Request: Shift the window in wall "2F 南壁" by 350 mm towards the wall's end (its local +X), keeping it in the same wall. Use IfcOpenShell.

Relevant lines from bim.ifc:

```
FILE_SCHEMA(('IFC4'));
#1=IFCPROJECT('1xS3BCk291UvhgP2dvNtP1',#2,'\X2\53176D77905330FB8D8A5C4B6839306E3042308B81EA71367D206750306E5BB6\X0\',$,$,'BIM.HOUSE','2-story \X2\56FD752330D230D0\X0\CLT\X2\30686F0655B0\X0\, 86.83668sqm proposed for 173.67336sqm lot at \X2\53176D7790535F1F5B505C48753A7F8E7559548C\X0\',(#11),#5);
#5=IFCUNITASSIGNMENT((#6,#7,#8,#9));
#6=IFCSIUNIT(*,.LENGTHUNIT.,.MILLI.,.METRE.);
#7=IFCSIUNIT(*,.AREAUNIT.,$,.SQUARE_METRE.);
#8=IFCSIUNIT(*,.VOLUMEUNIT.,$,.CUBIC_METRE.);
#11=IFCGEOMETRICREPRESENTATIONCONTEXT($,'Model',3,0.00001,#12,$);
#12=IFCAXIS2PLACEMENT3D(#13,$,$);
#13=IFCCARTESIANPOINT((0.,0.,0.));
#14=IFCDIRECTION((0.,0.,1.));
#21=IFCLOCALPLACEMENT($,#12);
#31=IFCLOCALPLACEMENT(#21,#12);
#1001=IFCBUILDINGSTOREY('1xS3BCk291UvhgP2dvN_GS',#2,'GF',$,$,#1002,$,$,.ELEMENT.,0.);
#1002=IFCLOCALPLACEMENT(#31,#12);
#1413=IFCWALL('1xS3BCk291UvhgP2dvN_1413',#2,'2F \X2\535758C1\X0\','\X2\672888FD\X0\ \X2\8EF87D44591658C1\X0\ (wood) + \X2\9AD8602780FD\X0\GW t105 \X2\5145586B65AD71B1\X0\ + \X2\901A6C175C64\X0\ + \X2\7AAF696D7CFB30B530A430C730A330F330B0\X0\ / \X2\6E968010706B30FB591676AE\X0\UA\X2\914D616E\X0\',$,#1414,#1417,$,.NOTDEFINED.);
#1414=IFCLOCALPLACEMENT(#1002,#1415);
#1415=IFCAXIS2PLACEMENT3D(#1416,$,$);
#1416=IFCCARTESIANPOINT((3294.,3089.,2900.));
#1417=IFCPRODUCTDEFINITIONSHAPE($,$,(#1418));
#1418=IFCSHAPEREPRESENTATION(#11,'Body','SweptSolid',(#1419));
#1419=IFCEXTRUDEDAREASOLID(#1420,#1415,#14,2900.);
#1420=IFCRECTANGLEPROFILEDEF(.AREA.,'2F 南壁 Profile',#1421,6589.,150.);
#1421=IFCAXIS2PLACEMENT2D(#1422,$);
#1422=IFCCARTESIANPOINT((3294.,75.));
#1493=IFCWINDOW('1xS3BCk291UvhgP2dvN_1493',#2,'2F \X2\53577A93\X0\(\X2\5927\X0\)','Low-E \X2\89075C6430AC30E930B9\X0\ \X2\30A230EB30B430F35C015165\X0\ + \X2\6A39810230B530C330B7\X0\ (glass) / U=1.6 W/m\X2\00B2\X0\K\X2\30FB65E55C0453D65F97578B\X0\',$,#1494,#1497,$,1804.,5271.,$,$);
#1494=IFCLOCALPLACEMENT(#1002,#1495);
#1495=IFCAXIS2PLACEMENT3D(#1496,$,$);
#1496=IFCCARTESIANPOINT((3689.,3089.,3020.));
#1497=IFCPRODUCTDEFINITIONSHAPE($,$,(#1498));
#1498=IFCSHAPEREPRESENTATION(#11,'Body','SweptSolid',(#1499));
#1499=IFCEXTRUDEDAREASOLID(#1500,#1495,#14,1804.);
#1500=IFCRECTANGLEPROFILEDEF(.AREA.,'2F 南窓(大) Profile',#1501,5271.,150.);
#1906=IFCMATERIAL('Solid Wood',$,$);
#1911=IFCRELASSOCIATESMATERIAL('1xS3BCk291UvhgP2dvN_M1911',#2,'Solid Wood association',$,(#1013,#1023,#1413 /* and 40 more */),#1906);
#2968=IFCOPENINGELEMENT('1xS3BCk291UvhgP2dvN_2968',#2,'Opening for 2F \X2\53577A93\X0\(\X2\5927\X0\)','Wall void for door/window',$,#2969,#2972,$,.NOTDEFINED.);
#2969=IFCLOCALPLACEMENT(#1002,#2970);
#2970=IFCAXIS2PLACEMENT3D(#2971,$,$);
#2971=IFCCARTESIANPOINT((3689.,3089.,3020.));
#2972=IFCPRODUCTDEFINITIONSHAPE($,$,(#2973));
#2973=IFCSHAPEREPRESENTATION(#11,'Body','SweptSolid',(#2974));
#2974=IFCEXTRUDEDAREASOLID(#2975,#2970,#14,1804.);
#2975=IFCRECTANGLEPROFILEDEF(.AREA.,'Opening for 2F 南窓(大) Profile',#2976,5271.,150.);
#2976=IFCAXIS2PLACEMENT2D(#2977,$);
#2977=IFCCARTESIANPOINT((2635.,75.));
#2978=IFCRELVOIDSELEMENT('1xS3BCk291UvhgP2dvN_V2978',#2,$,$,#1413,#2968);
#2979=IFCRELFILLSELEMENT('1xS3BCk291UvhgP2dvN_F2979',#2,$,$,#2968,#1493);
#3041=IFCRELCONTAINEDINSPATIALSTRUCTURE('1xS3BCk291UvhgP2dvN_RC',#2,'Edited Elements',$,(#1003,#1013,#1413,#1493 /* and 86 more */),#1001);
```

```python
import ifcopenshell
import ifcopenshell.api.geometry
import ifcopenshell.util.placement
import ifcopenshell.util.unit

model = ifcopenshell.open("bim.ifc")
unit_scale = ifcopenshell.util.unit.calculate_unit_scale(model)

window = model.by_guid("1xS3BCk291UvhgP2dvN_1493")
opening = window.FillsVoids[0].RelatingOpeningElement
wall = opening.VoidsElements[0].RelatingBuildingElement

wall_matrix = ifcopenshell.util.placement.get_local_placement(wall.ObjectPlacement)
shift = wall_matrix[:3, 0] * 0.35 / unit_scale
before = ifcopenshell.util.placement.get_local_placement(window.ObjectPlacement)[:3, 3].copy()

# The window is not placed relative to its opening, so move both.
for product in (opening, window):
    matrix = ifcopenshell.util.placement.get_local_placement(product.ObjectPlacement)
    matrix[:3, 3] += shift
    ifcopenshell.api.geometry.edit_object_placement(model, product=product, matrix=matrix, is_si=False)

after = ifcopenshell.util.placement.get_local_placement(window.ObjectPlacement)[:3, 3]
print("window moved by", (after - before).round(3) + 0.0)

model.write("bim_v2.ifc")
```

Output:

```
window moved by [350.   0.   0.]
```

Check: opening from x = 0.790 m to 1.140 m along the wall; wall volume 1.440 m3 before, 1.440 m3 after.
